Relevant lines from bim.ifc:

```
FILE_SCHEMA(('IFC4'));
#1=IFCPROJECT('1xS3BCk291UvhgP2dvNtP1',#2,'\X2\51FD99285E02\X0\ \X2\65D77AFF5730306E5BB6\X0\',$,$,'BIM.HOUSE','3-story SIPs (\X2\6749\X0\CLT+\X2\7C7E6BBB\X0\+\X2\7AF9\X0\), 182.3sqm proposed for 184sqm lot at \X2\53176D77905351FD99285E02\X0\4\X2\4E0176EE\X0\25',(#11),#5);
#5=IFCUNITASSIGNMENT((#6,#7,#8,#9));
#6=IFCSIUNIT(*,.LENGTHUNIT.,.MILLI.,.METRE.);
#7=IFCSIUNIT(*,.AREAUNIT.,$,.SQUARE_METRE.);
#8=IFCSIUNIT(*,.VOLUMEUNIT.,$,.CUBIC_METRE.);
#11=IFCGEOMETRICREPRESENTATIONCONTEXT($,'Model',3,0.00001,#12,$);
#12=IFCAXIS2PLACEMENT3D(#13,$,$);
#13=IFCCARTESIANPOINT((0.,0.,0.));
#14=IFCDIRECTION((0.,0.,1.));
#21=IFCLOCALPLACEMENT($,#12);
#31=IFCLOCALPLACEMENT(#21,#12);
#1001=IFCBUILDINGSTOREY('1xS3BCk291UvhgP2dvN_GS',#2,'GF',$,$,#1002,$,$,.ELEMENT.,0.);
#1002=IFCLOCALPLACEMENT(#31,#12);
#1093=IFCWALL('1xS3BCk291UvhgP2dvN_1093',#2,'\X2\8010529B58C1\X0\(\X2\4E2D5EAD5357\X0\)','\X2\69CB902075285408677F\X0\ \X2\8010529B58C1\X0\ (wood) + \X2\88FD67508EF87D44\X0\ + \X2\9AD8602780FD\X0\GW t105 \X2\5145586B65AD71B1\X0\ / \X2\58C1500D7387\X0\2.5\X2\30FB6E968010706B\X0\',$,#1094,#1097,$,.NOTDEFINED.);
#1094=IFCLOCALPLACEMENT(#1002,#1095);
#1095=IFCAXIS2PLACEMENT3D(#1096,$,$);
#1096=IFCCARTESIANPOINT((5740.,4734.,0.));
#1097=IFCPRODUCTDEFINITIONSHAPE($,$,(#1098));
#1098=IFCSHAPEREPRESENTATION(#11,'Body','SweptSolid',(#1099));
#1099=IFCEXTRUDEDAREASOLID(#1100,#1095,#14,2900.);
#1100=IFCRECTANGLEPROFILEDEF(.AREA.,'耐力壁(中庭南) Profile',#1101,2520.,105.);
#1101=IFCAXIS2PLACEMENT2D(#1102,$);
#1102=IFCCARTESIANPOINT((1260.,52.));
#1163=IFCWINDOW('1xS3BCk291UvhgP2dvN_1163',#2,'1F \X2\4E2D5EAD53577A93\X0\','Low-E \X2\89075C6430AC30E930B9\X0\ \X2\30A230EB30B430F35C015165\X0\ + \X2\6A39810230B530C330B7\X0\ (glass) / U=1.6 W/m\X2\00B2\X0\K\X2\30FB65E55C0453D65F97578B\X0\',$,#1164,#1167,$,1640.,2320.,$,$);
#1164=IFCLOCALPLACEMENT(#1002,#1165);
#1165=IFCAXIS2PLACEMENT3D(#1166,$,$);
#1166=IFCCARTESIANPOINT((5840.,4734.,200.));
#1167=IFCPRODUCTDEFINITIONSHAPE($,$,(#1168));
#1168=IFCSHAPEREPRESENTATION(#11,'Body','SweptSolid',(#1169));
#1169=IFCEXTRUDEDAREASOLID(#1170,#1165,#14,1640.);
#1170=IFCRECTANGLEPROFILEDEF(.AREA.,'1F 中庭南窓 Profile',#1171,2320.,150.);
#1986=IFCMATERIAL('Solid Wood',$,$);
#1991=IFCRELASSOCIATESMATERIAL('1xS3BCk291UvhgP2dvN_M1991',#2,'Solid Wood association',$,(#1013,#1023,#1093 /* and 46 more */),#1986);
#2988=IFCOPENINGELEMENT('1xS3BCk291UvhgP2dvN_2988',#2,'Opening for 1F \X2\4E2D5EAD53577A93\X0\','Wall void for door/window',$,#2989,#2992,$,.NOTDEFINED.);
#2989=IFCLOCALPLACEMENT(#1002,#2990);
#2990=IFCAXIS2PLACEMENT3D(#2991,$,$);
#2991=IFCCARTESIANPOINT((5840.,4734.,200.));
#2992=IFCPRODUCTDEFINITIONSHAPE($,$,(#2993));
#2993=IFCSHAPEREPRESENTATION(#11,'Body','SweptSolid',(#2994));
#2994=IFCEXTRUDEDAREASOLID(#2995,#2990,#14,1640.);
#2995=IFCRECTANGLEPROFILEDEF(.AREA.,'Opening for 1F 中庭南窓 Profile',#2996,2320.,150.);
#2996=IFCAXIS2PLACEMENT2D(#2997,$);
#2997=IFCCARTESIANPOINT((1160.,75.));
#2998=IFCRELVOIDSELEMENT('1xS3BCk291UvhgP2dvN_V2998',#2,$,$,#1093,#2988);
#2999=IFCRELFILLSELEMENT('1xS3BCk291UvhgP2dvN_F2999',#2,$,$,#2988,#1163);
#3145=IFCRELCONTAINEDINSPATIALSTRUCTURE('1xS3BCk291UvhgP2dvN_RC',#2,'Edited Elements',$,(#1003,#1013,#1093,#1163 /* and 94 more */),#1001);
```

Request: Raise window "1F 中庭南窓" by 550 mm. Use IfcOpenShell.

```python
import numpy as np
import ifcopenshell
import ifcopenshell.api.geometry
import ifcopenshell.util.placement
import ifcopenshell.util.unit

model = ifcopenshell.open("bim.ifc")
unit_scale = ifcopenshell.util.unit.calculate_unit_scale(model)

window = model.by_id(1163)
opening = window.FillsVoids[0].RelatingOpeningElement
dz = 0.55 / unit_scale

shift = np.array([0.0, 0.0, dz])
# The window is not placed relative to its opening, so move both.
for product in (opening, window):
    matrix = ifcopenshell.util.placement.get_local_placement(product.ObjectPlacement)
    matrix[:3, 3] += shift
    ifcopenshell.api.geometry.edit_object_placement(model, product=product, matrix=matrix, is_si=False)

print(f"moved by {dz * unit_scale:+.3f} m")

model.write("bim-out.ifc")
```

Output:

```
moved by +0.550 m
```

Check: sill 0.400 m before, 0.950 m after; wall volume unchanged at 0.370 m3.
